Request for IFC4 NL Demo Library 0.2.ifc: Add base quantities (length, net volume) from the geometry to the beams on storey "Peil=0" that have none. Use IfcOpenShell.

First a look at what the model holds.

```python
import ifcopenshell
import ifcopenshell.util.element
import ifcopenshell.util.unit

model = ifcopenshell.open("IFC4 NL Demo Library 0.2.ifc")
print(model.schema)
for unit_type in ("LENGTHUNIT", "AREAUNIT", "VOLUMEUNIT"):
    print(unit_type, ifcopenshell.util.unit.calculate_unit_scale(model, unit_type))
storey = next(s for s in model.by_type("IfcBuildingStorey") if s.Name == "Peil=0")
beams = [e for e in ifcopenshell.util.element.get_decomposition(storey) if e.is_a("IfcBeam")]
for e in sorted(beams, key=lambda e: e.id()):
    print(e.id(), e.is_a(), e.Name, list(ifcopenshell.util.element.get_psets(e, qtos_only=True)), sep=" | ")
```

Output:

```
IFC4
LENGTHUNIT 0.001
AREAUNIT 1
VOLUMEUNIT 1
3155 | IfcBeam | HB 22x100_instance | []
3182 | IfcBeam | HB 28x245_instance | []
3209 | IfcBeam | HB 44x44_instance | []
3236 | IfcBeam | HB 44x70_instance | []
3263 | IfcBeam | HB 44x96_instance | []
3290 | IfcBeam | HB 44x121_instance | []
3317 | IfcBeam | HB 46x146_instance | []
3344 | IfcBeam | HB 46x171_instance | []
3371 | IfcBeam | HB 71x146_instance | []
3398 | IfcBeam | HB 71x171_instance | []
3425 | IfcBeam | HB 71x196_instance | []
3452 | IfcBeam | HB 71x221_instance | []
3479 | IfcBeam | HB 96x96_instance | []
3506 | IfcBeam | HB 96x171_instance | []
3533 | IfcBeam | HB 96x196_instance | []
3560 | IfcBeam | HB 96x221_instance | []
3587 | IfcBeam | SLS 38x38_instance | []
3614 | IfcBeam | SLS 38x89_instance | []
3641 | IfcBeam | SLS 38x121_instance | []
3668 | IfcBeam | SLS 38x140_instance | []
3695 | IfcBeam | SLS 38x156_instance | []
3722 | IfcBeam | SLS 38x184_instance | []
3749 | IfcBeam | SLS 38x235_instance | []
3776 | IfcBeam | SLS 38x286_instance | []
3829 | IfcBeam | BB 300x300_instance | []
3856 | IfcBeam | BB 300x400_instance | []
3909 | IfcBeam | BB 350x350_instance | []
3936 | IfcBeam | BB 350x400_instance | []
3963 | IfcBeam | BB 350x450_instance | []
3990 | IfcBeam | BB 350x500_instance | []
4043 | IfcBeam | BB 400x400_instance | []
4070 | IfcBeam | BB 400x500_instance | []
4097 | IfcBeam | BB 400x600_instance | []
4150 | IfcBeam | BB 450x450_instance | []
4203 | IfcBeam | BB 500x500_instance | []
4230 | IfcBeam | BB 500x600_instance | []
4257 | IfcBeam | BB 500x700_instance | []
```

```python
import ifcopenshell
import ifcopenshell.api.pset
import ifcopenshell.geom
import ifcopenshell.util.element
import ifcopenshell.util.shape
import ifcopenshell.util.unit

model = ifcopenshell.open("IFC4 NL Demo Library 0.2.ifc")
unit_scale = ifcopenshell.util.unit.calculate_unit_scale(model)
volume_scale = ifcopenshell.util.unit.calculate_unit_scale(model, "VOLUMEUNIT")
settings = ifcopenshell.geom.settings()

storey = next(s for s in model.by_type("IfcBuildingStorey") if s.Name == "Peil=0")
beams = [e for e in ifcopenshell.util.element.get_decomposition(storey) if e.is_a("IfcBeam")]

for e in sorted(beams, key=lambda e: e.id()):
    if ifcopenshell.util.element.get_psets(e, qtos_only=True, should_inherit=False):
        continue
    # Geometry comes back in metres, in the element's own axes.
    shape = ifcopenshell.geom.create_shape(settings, e)
    values = {
        "Length": ifcopenshell.util.shape.get_max_xyz(shape.geometry) / unit_scale,
        "NetVolume": ifcopenshell.util.shape.get_volume(shape.geometry) / volume_scale,
    }
    qto = ifcopenshell.api.pset.add_qto(model, product=e, name="Qto_BeamBaseQuantities")
    ifcopenshell.api.pset.edit_qto(model, qto=qto, properties=values)
    print(e.id(), {k: round(v, 3) for k, v in values.items()})

model.write("IFC4 NL Demo Library 0.2_rev.ifc")
```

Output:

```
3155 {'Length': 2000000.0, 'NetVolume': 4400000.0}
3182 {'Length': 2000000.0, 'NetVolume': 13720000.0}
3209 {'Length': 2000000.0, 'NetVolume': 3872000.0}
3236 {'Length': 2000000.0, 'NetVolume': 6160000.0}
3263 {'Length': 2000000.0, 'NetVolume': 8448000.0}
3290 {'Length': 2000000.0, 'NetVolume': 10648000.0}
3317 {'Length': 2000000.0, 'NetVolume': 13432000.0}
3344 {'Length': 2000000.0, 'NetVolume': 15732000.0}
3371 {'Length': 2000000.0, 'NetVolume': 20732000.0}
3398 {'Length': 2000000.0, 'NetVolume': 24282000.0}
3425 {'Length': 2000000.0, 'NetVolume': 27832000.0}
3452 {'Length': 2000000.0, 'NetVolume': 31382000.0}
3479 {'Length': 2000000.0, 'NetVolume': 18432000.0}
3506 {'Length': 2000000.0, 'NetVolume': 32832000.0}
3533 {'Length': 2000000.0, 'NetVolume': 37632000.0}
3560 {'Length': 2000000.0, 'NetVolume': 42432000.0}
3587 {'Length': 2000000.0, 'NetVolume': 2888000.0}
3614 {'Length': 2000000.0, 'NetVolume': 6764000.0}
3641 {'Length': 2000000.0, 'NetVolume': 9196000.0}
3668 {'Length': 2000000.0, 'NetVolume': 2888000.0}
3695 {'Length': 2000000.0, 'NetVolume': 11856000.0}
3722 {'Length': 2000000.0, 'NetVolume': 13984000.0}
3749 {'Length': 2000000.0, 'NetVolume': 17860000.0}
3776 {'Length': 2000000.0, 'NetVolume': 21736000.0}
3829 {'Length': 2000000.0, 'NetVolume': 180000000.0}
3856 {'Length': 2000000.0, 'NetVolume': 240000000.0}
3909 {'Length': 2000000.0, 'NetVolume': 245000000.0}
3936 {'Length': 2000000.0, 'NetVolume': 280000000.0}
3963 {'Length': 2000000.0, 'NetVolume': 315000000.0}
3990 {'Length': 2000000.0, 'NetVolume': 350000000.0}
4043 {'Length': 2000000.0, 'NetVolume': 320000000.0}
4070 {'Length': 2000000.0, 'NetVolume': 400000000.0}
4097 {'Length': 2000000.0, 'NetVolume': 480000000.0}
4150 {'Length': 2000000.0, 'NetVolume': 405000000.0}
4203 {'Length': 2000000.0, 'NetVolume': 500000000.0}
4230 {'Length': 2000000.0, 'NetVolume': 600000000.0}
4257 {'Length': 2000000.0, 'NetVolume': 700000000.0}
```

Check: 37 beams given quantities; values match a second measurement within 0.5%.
